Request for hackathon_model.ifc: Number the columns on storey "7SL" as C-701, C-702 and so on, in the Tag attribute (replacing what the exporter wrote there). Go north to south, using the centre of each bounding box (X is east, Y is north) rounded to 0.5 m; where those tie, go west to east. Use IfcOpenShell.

First a look at what the model holds.

```python
import ifcopenshell
import ifcopenshell.util.element
import ifcopenshell.util.placement

model = ifcopenshell.open("hackathon_model.ifc")
print(model.schema)
storey = next(s for s in model.by_type("IfcBuildingStorey") if s.Name == "7SL")
columns = [e for e in ifcopenshell.util.element.get_decomposition(storey) if e.is_a("IfcColumn")]
for e in sorted(columns, key=lambda e: e.id()):
    origin = ifcopenshell.util.placement.get_local_placement(e.ObjectPlacement)[:3, 3]
    print(e.id(), e.Tag, e.Name, origin.round(2) + 0.0, sep=" | ")
```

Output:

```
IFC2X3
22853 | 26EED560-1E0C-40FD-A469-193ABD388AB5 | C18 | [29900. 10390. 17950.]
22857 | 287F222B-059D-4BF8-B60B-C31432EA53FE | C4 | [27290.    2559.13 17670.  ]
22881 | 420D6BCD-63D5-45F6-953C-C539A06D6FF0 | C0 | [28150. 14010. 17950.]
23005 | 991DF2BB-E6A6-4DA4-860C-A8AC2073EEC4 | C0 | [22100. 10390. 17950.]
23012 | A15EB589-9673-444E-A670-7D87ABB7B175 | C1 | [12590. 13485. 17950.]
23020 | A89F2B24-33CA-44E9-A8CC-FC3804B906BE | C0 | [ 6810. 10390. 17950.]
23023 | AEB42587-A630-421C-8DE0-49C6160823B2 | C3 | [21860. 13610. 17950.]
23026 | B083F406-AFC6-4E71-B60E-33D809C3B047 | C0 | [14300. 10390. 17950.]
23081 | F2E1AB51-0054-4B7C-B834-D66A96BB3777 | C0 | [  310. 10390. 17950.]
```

```python
import ifcopenshell
import ifcopenshell.geom
import ifcopenshell.util.element
import ifcopenshell.util.shape

model = ifcopenshell.open("hackathon_model.ifc")
settings = ifcopenshell.geom.settings()
settings.set("use-world-coords", True)


def centre(element):
    shape = ifcopenshell.geom.create_shape(settings, element)
    return ifcopenshell.util.shape.get_bbox_centroid(shape.geometry)


storey = next(s for s in model.by_type("IfcBuildingStorey") if s.Name == "7SL")
columns = [e for e in ifcopenshell.util.element.get_decomposition(storey) if e.is_a("IfcColumn")]

# Insertion points can sit at a corner or the storey origin, so sort by the geometry (in metres).
centres = {e: centre(e) for e in columns}
columns.sort(key=lambda e: (-round(centres[e][1] / 0.5), centres[e][0]))

for i, e in enumerate(columns, start=1):
    number = f"C-7{i:02d}"
    e.Tag = number
    print(e.id(), number)

model.write("hackathon_model_edited.ifc")
```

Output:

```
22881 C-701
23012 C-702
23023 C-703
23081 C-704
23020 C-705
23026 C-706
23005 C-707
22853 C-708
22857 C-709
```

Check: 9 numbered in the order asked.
